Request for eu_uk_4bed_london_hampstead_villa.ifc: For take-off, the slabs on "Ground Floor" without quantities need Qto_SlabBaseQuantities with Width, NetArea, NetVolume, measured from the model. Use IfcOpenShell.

First a look at what the model holds.

```python
import ifcopenshell
import ifcopenshell.util.element
import ifcopenshell.util.unit

model = ifcopenshell.open("eu_uk_4bed_london_hampstead_villa.ifc")
print(model.schema)
for unit_type in ("LENGTHUNIT", "AREAUNIT", "VOLUMEUNIT"):
    print(unit_type, ifcopenshell.util.unit.calculate_unit_scale(model, unit_type))
storey = next(s for s in model.by_type("IfcBuildingStorey") if s.Name == "Ground Floor")
slabs = [e for e in ifcopenshell.util.element.get_decomposition(storey) if e.is_a("IfcSlab")]
for e in sorted(slabs, key=lambda e: e.id()):
    print(e.id(), e.is_a(), e.Name, list(ifcopenshell.util.element.get_psets(e, qtos_only=True)), sep=" | ")
```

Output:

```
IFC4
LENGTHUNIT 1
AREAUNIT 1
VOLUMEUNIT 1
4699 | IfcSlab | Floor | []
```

```python
import ifcopenshell
import ifcopenshell.api.pset
import ifcopenshell.geom
import ifcopenshell.util.element
import ifcopenshell.util.shape
import ifcopenshell.util.unit

model = ifcopenshell.open("eu_uk_4bed_london_hampstead_villa.ifc")
unit_scale = ifcopenshell.util.unit.calculate_unit_scale(model)
area_scale = ifcopenshell.util.unit.calculate_unit_scale(model, "AREAUNIT")
volume_scale = ifcopenshell.util.unit.calculate_unit_scale(model, "VOLUMEUNIT")
settings = ifcopenshell.geom.settings()

storey = next(s for s in model.by_type("IfcBuildingStorey") if s.Name == "Ground Floor")
slabs = [e for e in ifcopenshell.util.element.get_decomposition(storey) if e.is_a("IfcSlab")]

for e in sorted(slabs, key=lambda e: e.id()):
    if ifcopenshell.util.element.get_psets(e, qtos_only=True, should_inherit=False):
        continue
    # Geometry comes back in metres, in the element's own axes.
    shape = ifcopenshell.geom.create_shape(settings, e)
    values = {
        "Width": ifcopenshell.util.shape.get_z(shape.geometry) / unit_scale,
        "NetArea": ifcopenshell.util.shape.get_footprint_area(shape.geometry) / area_scale,
        "NetVolume": ifcopenshell.util.shape.get_volume(shape.geometry) / volume_scale,
    }
    qto = ifcopenshell.api.pset.add_qto(model, product=e, name="Qto_SlabBaseQuantities")
    ifcopenshell.api.pset.edit_qto(model, qto=qto, properties=values)
    print(e.id(), {k: round(v, 3) for k, v in values.items()})

model.write("eu_uk_4bed_london_hampstead_villa_updated.ifc")
```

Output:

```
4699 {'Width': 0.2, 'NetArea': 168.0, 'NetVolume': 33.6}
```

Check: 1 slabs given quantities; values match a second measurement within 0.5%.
